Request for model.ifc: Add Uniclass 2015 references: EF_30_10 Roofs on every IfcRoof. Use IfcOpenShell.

First a look at what the model holds.

```python
import ifcopenshell

model = ifcopenshell.open("model.ifc")
print(model.schema)
print("classifications:", [c.Name for c in model.by_type("IfcClassification")])
for ifc_class in ("IfcDoor", "IfcRoof", "IfcStair", "IfcWall", "IfcWindow"):
    print(ifc_class, len(model.by_type(ifc_class)))
```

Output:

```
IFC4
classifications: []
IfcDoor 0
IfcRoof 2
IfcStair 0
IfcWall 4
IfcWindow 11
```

```python
import ifcopenshell
import ifcopenshell.api.classification

model = ifcopenshell.open("model.ifc")

system = ifcopenshell.api.classification.add_classification(model, classification="Uniclass 2015")

codes = {
    "IfcRoof": ("EF_30_10", "Roofs"),
}
for ifc_class, (code, name) in codes.items():
    products = model.by_type(ifc_class)
    ifcopenshell.api.classification.add_reference(
        model, products=products, classification=system, identification=code, name=name
    )
    print(code, len(products))

model.write("model-out.ifc")
```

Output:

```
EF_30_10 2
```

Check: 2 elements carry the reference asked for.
